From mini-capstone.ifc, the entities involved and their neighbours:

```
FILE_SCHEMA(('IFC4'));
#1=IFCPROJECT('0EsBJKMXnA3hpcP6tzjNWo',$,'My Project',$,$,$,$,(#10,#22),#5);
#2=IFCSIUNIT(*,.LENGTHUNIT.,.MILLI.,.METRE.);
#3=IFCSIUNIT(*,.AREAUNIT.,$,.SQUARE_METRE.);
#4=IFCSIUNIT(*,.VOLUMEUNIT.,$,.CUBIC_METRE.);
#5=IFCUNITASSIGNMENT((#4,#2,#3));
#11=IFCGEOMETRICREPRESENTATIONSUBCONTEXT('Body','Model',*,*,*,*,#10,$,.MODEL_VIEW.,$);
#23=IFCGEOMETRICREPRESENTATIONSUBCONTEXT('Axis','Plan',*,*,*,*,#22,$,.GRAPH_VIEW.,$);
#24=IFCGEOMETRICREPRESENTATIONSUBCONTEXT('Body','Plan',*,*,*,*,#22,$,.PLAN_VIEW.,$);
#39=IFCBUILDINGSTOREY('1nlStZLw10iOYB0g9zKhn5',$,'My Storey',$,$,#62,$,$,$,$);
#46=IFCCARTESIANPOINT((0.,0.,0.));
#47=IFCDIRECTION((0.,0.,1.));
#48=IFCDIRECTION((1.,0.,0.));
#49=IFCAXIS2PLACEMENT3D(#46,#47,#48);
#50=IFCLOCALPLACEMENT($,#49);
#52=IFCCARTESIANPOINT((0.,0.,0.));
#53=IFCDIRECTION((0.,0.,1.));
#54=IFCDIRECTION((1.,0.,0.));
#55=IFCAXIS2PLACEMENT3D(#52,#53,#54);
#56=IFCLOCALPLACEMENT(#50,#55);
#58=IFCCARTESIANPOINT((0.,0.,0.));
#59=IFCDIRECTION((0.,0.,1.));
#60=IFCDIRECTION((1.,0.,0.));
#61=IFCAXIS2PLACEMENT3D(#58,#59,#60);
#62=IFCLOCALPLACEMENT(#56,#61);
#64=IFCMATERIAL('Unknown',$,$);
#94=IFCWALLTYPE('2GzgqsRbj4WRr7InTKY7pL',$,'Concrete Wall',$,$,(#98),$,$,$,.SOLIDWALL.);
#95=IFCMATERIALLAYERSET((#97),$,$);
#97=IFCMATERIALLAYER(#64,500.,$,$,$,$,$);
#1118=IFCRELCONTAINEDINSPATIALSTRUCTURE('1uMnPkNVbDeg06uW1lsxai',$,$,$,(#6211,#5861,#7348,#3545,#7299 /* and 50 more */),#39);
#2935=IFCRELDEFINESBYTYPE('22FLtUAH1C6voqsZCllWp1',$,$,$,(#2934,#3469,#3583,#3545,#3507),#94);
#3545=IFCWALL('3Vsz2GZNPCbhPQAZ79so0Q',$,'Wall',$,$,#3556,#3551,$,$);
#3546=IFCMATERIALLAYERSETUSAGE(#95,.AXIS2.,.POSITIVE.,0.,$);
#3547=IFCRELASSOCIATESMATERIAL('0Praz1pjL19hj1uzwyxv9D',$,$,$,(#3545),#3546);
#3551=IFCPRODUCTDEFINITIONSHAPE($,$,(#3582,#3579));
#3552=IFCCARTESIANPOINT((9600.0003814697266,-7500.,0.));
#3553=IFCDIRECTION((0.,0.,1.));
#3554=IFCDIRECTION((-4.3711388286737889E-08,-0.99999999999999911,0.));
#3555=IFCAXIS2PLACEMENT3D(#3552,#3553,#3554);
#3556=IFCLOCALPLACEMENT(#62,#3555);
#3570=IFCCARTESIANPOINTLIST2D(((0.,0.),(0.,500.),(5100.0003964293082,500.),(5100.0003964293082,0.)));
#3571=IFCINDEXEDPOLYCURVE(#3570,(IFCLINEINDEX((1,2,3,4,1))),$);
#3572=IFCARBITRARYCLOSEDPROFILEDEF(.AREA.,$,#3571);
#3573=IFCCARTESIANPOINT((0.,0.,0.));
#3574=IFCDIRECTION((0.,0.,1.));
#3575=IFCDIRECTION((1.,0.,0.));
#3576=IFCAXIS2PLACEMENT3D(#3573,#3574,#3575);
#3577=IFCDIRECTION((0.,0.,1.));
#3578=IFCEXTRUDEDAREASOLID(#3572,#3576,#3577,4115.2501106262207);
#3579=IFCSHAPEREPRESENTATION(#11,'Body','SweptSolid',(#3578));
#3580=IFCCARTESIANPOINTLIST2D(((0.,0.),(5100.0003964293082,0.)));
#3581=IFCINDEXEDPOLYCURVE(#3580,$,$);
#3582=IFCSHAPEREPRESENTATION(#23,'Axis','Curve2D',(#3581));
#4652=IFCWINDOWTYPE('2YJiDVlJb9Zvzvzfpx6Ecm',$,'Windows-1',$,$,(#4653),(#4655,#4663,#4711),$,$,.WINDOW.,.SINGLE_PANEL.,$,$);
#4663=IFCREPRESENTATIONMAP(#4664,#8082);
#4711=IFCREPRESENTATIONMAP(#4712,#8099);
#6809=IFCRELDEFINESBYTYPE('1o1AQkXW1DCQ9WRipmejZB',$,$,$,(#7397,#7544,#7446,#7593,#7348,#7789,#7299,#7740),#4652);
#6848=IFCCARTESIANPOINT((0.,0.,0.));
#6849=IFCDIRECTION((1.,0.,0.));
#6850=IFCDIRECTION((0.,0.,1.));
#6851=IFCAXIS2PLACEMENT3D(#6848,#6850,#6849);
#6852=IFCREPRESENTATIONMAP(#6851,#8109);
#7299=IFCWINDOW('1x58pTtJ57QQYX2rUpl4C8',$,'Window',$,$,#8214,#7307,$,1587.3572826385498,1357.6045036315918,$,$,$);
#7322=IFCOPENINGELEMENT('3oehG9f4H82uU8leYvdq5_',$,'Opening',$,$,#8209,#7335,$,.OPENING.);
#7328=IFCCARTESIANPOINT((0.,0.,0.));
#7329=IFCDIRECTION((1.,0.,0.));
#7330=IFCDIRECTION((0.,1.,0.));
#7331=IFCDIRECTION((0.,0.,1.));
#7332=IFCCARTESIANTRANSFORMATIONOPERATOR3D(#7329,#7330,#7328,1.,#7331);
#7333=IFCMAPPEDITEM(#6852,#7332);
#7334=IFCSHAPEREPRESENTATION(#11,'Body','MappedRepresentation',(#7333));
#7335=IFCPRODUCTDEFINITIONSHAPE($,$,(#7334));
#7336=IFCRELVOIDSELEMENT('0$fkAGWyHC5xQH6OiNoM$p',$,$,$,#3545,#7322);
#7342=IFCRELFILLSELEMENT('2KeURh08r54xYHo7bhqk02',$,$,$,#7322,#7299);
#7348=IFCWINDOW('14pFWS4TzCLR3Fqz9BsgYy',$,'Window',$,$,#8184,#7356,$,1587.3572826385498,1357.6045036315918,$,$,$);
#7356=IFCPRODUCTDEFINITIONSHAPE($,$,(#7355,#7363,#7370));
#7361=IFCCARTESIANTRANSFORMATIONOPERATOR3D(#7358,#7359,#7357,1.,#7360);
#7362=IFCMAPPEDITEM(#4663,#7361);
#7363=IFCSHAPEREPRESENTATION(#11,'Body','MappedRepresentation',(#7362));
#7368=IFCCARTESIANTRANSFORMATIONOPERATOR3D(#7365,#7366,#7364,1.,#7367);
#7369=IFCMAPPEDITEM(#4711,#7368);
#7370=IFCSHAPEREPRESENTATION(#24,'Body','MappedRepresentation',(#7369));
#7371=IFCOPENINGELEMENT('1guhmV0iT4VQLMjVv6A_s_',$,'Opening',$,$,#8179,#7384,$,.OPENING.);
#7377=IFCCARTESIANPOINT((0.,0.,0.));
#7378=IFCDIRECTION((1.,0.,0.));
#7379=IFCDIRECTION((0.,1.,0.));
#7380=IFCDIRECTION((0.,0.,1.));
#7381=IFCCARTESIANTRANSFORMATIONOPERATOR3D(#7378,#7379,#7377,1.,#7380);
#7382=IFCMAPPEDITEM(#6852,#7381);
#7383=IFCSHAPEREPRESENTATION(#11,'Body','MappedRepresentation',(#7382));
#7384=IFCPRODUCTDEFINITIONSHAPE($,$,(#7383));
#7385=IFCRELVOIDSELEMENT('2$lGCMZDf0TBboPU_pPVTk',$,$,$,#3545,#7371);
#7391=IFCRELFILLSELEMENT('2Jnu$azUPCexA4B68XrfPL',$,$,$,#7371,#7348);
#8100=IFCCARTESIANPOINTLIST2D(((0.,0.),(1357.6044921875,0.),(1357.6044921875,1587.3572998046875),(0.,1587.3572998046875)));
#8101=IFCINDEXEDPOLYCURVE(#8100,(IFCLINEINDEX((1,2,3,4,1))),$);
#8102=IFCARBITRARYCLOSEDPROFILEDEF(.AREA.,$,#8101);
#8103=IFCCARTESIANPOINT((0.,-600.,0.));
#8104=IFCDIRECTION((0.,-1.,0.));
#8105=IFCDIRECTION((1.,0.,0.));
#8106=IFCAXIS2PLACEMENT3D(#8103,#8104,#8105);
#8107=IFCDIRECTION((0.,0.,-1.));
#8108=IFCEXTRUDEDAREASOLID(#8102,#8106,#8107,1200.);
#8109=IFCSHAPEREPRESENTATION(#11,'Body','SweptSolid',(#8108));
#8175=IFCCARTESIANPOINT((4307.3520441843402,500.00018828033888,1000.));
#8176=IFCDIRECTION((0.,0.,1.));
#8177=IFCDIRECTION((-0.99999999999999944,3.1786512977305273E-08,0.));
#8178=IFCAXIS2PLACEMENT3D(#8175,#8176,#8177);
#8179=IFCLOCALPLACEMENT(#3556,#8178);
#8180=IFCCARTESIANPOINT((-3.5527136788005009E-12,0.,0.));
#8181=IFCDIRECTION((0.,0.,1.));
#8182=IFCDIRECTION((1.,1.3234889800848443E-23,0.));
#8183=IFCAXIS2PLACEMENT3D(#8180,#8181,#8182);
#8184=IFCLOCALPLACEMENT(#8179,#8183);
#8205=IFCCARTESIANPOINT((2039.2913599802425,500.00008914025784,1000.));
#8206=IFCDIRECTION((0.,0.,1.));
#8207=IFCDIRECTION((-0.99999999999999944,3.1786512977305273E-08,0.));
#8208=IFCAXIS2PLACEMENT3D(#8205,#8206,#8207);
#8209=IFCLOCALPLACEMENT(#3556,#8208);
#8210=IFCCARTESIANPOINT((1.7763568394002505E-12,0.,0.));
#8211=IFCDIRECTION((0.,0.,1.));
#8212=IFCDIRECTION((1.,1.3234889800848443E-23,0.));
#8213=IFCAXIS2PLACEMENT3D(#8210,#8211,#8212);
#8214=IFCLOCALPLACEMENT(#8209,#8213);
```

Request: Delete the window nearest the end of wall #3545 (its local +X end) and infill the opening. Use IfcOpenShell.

```python
import ifcopenshell
import ifcopenshell.api.feature
import ifcopenshell.api.root
import ifcopenshell.geom
import ifcopenshell.util.shape

model = ifcopenshell.open("mini-capstone.ifc")
settings = ifcopenshell.geom.settings()


def volume(element):
    """Net volume in cubic metres, openings subtracted."""
    shape = ifcopenshell.geom.create_shape(settings, element)
    return ifcopenshell.util.shape.get_volume(shape.geometry)


window = model.by_guid("14pFWS4TzCLR3Fqz9BsgYy")
opening = window.FillsVoids[0].RelatingOpeningElement
wall = opening.VoidsElements[0].RelatingBuildingElement
before = volume(wall)

ifcopenshell.api.root.remove_product(model, product=window)
ifcopenshell.api.feature.remove_feature(model, feature=opening)

after = volume(wall)

print(f"wall volume {before:.3f} -> {after:.3f} m3")

model.write("mini-capstone-out.ifc")
```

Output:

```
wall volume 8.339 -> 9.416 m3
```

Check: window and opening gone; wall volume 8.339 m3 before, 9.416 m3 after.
